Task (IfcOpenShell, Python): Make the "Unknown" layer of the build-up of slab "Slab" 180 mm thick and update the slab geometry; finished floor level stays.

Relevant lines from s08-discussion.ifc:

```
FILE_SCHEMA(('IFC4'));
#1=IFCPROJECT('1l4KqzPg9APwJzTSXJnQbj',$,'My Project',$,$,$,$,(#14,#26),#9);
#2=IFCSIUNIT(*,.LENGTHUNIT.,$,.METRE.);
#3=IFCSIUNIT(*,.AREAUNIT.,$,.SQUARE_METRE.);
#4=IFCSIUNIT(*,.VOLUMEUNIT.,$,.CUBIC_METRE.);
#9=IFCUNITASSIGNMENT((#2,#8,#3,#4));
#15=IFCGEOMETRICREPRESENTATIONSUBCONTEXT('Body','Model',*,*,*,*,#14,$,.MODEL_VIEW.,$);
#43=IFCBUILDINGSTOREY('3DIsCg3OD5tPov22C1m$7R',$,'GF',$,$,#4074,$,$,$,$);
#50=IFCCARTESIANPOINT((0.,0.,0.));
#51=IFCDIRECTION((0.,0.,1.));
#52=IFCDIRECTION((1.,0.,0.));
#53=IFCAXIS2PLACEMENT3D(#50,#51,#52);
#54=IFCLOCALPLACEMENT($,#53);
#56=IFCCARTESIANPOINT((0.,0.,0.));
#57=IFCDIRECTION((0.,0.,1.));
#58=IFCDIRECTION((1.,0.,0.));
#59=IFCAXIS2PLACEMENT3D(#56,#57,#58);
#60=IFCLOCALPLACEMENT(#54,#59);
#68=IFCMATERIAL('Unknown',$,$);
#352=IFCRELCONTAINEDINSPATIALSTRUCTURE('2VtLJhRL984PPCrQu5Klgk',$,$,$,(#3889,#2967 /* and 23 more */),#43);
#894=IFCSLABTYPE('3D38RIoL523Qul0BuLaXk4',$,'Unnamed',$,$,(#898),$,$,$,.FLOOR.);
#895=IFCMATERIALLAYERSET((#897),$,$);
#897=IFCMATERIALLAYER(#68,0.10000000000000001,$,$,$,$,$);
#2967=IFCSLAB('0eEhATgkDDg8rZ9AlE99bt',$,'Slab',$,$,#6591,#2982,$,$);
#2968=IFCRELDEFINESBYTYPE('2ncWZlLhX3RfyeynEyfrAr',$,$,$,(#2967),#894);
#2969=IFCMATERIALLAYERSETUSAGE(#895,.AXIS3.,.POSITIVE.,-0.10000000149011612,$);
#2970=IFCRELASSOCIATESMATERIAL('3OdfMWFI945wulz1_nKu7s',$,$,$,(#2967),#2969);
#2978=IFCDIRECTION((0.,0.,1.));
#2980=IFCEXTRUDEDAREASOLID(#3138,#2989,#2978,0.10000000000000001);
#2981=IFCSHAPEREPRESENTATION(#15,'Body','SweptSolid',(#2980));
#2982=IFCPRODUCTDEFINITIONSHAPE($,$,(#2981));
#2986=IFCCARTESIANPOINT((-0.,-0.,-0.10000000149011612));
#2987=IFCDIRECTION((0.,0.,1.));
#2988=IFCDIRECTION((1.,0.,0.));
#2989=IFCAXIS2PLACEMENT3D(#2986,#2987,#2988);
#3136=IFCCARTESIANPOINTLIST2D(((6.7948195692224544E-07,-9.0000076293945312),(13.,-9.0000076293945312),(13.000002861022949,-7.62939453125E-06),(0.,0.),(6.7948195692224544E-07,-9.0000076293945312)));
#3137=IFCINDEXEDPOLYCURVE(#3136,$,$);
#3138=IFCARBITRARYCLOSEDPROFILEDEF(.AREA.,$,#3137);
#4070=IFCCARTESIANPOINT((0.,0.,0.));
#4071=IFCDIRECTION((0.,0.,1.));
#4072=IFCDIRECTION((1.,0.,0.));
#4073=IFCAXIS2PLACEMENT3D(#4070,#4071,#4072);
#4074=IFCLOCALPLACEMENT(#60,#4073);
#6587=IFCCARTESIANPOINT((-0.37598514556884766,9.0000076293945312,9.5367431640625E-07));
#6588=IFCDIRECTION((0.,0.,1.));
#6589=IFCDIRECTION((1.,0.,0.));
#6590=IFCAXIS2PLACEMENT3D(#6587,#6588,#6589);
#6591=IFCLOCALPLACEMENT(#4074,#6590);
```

```python
import ifcopenshell
import ifcopenshell.util.element
import ifcopenshell.util.representation

model = ifcopenshell.open("s08-discussion.ifc")

layer_set = model.by_id(895)
layer = next(l for l in layer_set.MaterialLayers if l.Material and l.Material.Name == "Unknown")
change = 0.18 - layer.LayerThickness
layer.LayerThickness += change

# Geometry does not follow the layer set by itself.
slabs = [e for e in ifcopenshell.util.element.get_elements_by_material(model, layer_set) if e.is_a("IfcSlab")]
for slab in sorted(slabs, key=lambda e: e.id()):
    body = ifcopenshell.util.representation.get_representation(slab, "Model", "Body")
    solid = body.Items[0]
    old_depth = solid.Depth
    solid.Depth += change
    # Extruded upwards: lower the start of the extrusion so the top stays.
    x, y, z = solid.Position.Location.Coordinates
    solid.Position.Location = model.createIfcCartesianPoint((x, y, z - change))
    print(slab.id(), f"{old_depth:g} -> {solid.Depth:g}")

# The layers are counted up from the underside, which has moved.
for usage in {ifcopenshell.util.element.get_material(slab) for slab in slabs}:
    usage.OffsetFromReferenceLine -= change

model.write("s08-discussion_v2.ifc")
```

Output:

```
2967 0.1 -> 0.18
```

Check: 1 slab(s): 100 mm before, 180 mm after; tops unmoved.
